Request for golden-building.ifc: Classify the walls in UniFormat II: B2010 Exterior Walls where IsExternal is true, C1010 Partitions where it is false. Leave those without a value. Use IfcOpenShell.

First a look at what the model holds.

```python
import ifcopenshell
import ifcopenshell.util.element

model = ifcopenshell.open("golden-building.ifc")
print(model.schema)
print("classifications:", [c.Name for c in model.by_type("IfcClassification")])
values = [ifcopenshell.util.element.get_pset(e, "Pset_WallCommon", "IsExternal") for e in model.by_type("IfcWall")]
for value in (True, False, None):
    print("IsExternal", value, values.count(value))
```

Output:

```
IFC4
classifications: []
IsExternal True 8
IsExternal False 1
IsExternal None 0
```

```python
import ifcopenshell
import ifcopenshell.api.classification
import ifcopenshell.util.element

model = ifcopenshell.open("golden-building.ifc")

system = ifcopenshell.api.classification.add_classification(model, classification="UniFormat II")

walls = model.by_type("IfcWall")
external = {e: ifcopenshell.util.element.get_pset(e, "Pset_WallCommon", "IsExternal") for e in walls}
for flag, code, name in ((True, "B2010", "Exterior Walls"), (False, "C1010", "Partitions")):
    products = [e for e in walls if external[e] is flag]
    ifcopenshell.api.classification.add_reference(
        model, products=products, classification=system, identification=code, name=name
    )
    print(code, len(products))

model.write("golden-building-out.ifc")
```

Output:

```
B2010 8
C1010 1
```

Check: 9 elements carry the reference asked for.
